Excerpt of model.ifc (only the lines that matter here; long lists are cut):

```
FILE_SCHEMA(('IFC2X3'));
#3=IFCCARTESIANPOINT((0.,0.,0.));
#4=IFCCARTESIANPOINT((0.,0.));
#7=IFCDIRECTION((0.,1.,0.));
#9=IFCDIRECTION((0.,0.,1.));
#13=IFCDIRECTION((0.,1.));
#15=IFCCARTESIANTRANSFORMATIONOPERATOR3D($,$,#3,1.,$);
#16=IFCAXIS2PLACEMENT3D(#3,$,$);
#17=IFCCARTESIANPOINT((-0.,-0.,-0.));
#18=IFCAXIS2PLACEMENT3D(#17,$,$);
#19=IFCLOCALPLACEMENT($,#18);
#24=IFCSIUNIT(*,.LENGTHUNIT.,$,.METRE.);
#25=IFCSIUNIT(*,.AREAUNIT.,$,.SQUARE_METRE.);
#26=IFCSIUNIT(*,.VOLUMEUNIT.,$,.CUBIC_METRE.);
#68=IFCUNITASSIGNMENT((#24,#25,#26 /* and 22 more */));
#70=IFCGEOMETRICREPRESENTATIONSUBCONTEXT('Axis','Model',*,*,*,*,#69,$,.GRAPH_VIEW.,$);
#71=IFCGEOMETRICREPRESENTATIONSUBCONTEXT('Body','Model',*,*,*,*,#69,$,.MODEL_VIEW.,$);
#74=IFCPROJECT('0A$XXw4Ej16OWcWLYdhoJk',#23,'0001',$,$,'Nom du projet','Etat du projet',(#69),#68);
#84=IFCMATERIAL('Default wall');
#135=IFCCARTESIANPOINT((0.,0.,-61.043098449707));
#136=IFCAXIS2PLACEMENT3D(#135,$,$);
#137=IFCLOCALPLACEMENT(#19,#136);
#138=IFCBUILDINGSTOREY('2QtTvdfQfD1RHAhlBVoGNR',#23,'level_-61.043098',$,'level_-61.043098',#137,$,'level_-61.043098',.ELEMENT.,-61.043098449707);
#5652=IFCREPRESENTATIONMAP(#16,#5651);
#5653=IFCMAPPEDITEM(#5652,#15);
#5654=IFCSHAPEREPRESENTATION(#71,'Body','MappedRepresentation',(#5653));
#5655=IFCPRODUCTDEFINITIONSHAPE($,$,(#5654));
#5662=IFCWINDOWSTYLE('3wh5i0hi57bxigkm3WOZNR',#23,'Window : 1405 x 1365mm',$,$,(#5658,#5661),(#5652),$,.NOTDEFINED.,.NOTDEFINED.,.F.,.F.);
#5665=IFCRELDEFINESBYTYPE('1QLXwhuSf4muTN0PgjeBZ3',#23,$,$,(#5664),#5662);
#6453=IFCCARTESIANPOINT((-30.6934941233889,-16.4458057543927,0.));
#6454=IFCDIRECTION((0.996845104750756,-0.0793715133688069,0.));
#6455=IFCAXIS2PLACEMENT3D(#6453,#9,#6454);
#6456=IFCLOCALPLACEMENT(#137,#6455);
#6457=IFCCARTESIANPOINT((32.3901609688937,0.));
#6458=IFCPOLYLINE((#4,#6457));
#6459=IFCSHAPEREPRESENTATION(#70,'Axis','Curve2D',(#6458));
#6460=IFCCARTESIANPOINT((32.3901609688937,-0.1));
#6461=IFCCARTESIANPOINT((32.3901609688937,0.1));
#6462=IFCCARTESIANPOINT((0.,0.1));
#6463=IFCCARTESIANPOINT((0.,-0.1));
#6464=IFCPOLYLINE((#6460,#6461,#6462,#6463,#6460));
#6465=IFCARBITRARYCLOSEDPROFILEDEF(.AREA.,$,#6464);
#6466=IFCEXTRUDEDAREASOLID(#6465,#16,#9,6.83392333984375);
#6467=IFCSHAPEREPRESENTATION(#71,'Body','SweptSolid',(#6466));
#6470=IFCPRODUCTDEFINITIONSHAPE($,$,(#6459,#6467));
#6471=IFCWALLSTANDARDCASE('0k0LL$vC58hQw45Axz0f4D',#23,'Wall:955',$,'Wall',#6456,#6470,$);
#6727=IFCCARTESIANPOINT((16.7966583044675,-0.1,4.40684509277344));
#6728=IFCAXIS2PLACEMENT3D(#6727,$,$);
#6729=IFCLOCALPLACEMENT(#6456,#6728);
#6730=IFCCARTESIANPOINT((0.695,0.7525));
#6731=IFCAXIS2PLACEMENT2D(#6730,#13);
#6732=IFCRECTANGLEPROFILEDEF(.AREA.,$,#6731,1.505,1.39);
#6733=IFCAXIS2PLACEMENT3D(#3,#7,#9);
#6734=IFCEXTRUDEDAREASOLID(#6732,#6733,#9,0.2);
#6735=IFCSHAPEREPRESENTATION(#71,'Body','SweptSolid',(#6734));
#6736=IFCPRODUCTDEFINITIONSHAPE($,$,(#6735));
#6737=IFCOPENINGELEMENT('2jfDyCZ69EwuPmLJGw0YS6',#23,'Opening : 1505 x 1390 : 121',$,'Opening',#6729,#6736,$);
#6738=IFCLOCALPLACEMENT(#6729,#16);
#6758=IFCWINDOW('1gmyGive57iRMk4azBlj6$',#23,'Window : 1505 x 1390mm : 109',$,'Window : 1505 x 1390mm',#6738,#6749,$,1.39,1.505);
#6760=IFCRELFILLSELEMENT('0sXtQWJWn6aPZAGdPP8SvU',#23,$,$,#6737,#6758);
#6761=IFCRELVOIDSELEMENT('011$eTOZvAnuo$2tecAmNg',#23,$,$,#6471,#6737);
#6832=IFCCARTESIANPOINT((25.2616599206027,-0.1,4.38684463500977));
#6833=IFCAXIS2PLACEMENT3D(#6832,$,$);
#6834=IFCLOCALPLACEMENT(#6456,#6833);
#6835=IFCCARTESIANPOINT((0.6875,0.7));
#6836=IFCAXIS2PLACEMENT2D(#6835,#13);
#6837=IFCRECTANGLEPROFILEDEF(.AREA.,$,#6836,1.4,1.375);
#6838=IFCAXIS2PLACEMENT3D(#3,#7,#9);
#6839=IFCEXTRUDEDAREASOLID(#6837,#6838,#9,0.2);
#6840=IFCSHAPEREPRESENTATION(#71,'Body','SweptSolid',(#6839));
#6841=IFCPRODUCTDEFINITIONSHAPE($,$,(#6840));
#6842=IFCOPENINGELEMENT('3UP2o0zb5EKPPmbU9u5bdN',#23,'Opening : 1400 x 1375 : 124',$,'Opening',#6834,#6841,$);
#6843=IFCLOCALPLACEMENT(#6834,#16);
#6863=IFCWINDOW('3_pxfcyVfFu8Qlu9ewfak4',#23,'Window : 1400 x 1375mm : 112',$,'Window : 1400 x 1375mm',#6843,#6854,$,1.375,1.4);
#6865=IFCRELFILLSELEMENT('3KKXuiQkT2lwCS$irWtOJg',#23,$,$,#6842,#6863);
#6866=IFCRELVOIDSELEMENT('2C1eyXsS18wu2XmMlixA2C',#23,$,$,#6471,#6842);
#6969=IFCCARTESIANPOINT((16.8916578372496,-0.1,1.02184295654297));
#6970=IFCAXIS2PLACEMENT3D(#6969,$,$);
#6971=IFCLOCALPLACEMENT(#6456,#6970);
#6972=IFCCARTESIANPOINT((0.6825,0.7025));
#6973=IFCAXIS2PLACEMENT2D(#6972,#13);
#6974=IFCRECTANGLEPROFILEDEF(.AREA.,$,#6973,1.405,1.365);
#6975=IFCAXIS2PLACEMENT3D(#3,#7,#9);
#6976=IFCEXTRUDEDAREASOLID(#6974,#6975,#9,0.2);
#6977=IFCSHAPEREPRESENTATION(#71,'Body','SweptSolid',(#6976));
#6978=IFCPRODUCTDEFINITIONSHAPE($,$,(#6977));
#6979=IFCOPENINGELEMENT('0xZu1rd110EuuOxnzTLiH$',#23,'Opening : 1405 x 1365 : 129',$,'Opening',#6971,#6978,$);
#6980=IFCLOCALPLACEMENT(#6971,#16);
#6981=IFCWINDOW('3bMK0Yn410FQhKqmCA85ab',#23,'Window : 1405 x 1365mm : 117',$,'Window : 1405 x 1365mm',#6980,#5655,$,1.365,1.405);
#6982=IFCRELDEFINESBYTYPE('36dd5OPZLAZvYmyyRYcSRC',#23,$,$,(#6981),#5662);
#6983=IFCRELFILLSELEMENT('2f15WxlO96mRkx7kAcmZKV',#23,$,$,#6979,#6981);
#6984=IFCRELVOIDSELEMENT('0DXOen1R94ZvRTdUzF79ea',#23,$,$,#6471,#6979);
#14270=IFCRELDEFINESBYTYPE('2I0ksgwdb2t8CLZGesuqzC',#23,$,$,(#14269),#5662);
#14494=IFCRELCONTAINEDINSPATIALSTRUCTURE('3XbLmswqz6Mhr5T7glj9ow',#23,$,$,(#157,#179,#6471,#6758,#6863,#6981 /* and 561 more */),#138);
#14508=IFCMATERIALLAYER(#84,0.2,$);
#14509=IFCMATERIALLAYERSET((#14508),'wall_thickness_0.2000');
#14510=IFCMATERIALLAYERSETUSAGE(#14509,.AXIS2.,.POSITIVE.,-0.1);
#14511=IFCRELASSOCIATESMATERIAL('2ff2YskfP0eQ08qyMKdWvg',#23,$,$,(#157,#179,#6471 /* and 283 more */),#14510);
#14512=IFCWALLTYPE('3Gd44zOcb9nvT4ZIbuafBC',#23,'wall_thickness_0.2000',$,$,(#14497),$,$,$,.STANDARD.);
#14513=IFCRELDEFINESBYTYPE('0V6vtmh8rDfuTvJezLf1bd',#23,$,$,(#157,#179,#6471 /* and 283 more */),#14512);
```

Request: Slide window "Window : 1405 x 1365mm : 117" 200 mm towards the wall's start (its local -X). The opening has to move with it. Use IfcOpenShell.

```python
import ifcopenshell
import ifcopenshell.api.geometry
import ifcopenshell.util.placement
import ifcopenshell.util.unit

model = ifcopenshell.open("model.ifc")
unit_scale = ifcopenshell.util.unit.calculate_unit_scale(model)

window = model.by_id(6981)
opening = window.FillsVoids[0].RelatingOpeningElement
wall = opening.VoidsElements[0].RelatingBuildingElement

wall_matrix = ifcopenshell.util.placement.get_local_placement(wall.ObjectPlacement)
shift = wall_matrix[:3, 0] * -0.2 / unit_scale
before = ifcopenshell.util.placement.get_local_placement(window.ObjectPlacement)[:3, 3].copy()

# The window is placed relative to its opening, so it follows when the opening moves.
matrix = ifcopenshell.util.placement.get_local_placement(opening.ObjectPlacement)
matrix[:3, 3] += shift
ifcopenshell.api.geometry.edit_object_placement(
    model, product=opening, matrix=matrix, is_si=False, should_transform_children=True
)

after = ifcopenshell.util.placement.get_local_placement(window.ObjectPlacement)[:3, 3]
print("window moved by", (after - before).round(3) + 0.0)

model.write("model_rev.ifc")
```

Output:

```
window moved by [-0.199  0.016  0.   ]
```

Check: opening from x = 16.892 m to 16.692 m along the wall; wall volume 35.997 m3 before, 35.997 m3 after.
